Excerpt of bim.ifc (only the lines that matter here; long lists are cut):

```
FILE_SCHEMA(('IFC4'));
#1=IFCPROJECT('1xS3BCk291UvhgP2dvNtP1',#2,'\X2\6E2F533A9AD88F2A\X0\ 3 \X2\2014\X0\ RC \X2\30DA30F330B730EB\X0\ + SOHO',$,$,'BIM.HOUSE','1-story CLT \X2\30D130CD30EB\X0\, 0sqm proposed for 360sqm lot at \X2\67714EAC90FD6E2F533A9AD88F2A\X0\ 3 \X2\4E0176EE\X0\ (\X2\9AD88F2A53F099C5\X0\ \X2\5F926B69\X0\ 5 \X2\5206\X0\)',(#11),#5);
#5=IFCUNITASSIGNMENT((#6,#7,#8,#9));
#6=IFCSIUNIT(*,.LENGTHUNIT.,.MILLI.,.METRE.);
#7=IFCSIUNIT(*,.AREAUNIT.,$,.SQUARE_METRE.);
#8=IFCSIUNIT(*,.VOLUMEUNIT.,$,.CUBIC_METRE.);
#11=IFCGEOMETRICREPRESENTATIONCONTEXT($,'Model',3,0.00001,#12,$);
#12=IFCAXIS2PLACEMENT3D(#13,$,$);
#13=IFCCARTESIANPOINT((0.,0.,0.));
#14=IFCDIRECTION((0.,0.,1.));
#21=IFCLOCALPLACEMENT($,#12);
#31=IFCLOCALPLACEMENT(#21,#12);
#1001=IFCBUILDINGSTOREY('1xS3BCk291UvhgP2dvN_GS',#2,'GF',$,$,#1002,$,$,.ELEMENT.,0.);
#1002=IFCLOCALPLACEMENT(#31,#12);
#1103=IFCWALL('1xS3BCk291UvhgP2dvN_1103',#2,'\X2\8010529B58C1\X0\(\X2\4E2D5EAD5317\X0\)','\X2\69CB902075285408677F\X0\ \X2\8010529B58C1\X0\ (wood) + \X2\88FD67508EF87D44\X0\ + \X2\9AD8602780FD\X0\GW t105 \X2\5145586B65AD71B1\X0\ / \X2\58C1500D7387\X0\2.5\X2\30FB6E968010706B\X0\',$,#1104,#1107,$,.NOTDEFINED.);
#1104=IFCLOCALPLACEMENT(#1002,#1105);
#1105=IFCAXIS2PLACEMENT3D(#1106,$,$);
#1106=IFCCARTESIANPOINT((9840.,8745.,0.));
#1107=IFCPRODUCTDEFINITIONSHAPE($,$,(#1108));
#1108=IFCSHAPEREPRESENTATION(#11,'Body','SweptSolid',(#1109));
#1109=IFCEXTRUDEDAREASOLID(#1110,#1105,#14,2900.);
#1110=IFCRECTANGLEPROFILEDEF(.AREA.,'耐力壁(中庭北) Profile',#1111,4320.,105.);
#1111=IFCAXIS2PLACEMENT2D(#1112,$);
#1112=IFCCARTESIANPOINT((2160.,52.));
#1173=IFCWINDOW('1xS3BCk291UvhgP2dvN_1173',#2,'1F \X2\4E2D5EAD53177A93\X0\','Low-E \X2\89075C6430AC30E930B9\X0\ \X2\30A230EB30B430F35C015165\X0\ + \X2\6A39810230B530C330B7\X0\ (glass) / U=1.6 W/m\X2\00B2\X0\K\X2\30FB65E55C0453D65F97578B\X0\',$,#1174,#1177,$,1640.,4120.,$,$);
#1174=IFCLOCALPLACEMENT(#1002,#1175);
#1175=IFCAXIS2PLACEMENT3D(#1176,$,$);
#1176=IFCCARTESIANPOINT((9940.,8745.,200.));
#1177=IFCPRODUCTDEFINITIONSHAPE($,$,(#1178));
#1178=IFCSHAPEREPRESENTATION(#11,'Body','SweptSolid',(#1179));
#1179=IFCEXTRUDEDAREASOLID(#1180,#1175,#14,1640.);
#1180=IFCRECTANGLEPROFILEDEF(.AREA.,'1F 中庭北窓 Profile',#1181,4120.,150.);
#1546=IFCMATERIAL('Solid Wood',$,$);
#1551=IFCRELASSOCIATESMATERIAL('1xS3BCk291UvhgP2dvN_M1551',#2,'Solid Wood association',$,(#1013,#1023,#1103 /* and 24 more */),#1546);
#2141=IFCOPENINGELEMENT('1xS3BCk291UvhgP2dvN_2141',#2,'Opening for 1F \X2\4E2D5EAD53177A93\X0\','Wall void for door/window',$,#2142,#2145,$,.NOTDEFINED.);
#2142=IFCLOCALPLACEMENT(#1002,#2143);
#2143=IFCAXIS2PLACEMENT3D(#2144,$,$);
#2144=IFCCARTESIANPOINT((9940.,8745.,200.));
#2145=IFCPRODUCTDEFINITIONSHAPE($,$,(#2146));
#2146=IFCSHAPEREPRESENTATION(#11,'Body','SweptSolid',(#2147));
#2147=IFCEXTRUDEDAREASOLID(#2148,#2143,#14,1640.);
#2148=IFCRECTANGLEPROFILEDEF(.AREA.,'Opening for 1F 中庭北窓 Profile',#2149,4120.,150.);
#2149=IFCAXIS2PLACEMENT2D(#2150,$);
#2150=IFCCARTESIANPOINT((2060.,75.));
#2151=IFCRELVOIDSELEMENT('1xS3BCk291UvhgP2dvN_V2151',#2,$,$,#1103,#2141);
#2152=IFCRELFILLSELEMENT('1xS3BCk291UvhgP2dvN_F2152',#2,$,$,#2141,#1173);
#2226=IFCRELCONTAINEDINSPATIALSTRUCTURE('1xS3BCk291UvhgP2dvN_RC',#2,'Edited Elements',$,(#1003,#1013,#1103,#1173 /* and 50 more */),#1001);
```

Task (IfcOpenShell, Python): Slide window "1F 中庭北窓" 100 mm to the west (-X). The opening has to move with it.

```python
import ifcopenshell
import ifcopenshell.api.geometry
import ifcopenshell.util.placement

model = ifcopenshell.open("bim.ifc")

window = model.by_guid("1xS3BCk291UvhgP2dvN_1173")
opening = window.FillsVoids[0].RelatingOpeningElement
wall = opening.VoidsElements[0].RelatingBuildingElement

wall_matrix = ifcopenshell.util.placement.get_local_placement(wall.ObjectPlacement)
shift = wall_matrix[:3, 0] * -100.0
before = ifcopenshell.util.placement.get_local_placement(window.ObjectPlacement)[:3, 3].copy()

# The window is not placed relative to its opening, so move both.
for product in (opening, window):
    matrix = ifcopenshell.util.placement.get_local_placement(product.ObjectPlacement)
    matrix[:3, 3] += shift
    ifcopenshell.api.geometry.edit_object_placement(model, product=product, matrix=matrix, is_si=False)

after = ifcopenshell.util.placement.get_local_placement(window.ObjectPlacement)[:3, 3]
print("window moved by", (after - before).round(3) + 0.0)

model.write("bim_edited.ifc")
```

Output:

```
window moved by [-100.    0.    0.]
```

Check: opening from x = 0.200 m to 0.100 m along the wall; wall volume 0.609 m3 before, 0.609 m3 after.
